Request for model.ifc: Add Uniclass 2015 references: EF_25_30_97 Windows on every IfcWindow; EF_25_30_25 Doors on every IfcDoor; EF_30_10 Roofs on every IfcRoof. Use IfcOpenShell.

First a look at what the model holds.

```python
import ifcopenshell

model = ifcopenshell.open("model.ifc")
print(model.schema)
print("classifications:", [c.Name for c in model.by_type("IfcClassification")])
for ifc_class in ("IfcDoor", "IfcRoof", "IfcStair", "IfcWall", "IfcWindow"):
    print(ifc_class, len(model.by_type(ifc_class)))
```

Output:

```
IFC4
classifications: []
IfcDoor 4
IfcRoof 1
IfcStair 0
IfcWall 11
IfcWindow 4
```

```python
import ifcopenshell
import ifcopenshell.api.classification

model = ifcopenshell.open("model.ifc")

system = ifcopenshell.api.classification.add_classification(model, classification="Uniclass 2015")

codes = {
    "IfcWindow": ("EF_25_30_97", "Windows"),
    "IfcDoor": ("EF_25_30_25", "Doors"),
    "IfcRoof": ("EF_30_10", "Roofs"),
}
for ifc_class, (code, name) in codes.items():
    products = model.by_type(ifc_class)
    ifcopenshell.api.classification.add_reference(
        model, products=products, classification=system, identification=code, name=name
    )
    print(code, len(products))

model.write("model_rev.ifc")
```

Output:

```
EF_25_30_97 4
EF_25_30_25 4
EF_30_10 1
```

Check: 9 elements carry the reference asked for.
